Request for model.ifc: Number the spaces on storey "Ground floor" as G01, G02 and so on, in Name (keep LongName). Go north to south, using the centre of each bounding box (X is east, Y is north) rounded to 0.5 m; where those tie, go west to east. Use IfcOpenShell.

First a look at what the model holds.

```python
import ifcopenshell
import ifcopenshell.util.element
import ifcopenshell.util.placement

model = ifcopenshell.open("model.ifc")
print(model.schema)
storey = next(s for s in model.by_type("IfcBuildingStorey") if s.Name == "Ground floor")
spaces = [e for e in ifcopenshell.util.element.get_decomposition(storey) if e.is_a("IfcSpace")]
for e in sorted(spaces, key=lambda e: e.id()):
    origin = ifcopenshell.util.placement.get_local_placement(e.ObjectPlacement)[:3, 3]
    print(e.id(), e.Name, e.LongName, origin.round(2) + 0.0, sep=" | ")
```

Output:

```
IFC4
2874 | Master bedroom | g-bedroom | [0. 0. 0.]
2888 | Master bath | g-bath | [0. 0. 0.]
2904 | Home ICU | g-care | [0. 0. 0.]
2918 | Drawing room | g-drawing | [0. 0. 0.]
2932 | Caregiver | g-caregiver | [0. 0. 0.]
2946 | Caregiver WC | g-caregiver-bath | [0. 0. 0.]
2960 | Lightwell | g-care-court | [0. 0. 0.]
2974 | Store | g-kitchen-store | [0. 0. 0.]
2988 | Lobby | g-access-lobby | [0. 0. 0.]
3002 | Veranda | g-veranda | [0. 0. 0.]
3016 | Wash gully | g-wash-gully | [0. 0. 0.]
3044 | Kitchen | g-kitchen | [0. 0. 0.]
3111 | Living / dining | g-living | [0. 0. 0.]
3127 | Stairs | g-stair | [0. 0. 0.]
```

```python
import ifcopenshell
import ifcopenshell.geom
import ifcopenshell.util.element
import ifcopenshell.util.shape

model = ifcopenshell.open("model.ifc")
settings = ifcopenshell.geom.settings()
settings.set("use-world-coords", True)


def centre(element):
    shape = ifcopenshell.geom.create_shape(settings, element)
    return ifcopenshell.util.shape.get_bbox_centroid(shape.geometry)


storey = next(s for s in model.by_type("IfcBuildingStorey") if s.Name == "Ground floor")
spaces = [e for e in ifcopenshell.util.element.get_decomposition(storey) if e.is_a("IfcSpace")]

# Insertion points can sit at a corner or the storey origin, so sort by the geometry (in metres).
centres = {e: centre(e) for e in spaces}
spaces.sort(key=lambda e: (-round(centres[e][1] / 0.5), centres[e][0]))

for i, e in enumerate(spaces, start=1):
    number = f"G{i:02d}"
    e.Name = number
    print(e.id(), number)

model.write("model_v2.ifc")
```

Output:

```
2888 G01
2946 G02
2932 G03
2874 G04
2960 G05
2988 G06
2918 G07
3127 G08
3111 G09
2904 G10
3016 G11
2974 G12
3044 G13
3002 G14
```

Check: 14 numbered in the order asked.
